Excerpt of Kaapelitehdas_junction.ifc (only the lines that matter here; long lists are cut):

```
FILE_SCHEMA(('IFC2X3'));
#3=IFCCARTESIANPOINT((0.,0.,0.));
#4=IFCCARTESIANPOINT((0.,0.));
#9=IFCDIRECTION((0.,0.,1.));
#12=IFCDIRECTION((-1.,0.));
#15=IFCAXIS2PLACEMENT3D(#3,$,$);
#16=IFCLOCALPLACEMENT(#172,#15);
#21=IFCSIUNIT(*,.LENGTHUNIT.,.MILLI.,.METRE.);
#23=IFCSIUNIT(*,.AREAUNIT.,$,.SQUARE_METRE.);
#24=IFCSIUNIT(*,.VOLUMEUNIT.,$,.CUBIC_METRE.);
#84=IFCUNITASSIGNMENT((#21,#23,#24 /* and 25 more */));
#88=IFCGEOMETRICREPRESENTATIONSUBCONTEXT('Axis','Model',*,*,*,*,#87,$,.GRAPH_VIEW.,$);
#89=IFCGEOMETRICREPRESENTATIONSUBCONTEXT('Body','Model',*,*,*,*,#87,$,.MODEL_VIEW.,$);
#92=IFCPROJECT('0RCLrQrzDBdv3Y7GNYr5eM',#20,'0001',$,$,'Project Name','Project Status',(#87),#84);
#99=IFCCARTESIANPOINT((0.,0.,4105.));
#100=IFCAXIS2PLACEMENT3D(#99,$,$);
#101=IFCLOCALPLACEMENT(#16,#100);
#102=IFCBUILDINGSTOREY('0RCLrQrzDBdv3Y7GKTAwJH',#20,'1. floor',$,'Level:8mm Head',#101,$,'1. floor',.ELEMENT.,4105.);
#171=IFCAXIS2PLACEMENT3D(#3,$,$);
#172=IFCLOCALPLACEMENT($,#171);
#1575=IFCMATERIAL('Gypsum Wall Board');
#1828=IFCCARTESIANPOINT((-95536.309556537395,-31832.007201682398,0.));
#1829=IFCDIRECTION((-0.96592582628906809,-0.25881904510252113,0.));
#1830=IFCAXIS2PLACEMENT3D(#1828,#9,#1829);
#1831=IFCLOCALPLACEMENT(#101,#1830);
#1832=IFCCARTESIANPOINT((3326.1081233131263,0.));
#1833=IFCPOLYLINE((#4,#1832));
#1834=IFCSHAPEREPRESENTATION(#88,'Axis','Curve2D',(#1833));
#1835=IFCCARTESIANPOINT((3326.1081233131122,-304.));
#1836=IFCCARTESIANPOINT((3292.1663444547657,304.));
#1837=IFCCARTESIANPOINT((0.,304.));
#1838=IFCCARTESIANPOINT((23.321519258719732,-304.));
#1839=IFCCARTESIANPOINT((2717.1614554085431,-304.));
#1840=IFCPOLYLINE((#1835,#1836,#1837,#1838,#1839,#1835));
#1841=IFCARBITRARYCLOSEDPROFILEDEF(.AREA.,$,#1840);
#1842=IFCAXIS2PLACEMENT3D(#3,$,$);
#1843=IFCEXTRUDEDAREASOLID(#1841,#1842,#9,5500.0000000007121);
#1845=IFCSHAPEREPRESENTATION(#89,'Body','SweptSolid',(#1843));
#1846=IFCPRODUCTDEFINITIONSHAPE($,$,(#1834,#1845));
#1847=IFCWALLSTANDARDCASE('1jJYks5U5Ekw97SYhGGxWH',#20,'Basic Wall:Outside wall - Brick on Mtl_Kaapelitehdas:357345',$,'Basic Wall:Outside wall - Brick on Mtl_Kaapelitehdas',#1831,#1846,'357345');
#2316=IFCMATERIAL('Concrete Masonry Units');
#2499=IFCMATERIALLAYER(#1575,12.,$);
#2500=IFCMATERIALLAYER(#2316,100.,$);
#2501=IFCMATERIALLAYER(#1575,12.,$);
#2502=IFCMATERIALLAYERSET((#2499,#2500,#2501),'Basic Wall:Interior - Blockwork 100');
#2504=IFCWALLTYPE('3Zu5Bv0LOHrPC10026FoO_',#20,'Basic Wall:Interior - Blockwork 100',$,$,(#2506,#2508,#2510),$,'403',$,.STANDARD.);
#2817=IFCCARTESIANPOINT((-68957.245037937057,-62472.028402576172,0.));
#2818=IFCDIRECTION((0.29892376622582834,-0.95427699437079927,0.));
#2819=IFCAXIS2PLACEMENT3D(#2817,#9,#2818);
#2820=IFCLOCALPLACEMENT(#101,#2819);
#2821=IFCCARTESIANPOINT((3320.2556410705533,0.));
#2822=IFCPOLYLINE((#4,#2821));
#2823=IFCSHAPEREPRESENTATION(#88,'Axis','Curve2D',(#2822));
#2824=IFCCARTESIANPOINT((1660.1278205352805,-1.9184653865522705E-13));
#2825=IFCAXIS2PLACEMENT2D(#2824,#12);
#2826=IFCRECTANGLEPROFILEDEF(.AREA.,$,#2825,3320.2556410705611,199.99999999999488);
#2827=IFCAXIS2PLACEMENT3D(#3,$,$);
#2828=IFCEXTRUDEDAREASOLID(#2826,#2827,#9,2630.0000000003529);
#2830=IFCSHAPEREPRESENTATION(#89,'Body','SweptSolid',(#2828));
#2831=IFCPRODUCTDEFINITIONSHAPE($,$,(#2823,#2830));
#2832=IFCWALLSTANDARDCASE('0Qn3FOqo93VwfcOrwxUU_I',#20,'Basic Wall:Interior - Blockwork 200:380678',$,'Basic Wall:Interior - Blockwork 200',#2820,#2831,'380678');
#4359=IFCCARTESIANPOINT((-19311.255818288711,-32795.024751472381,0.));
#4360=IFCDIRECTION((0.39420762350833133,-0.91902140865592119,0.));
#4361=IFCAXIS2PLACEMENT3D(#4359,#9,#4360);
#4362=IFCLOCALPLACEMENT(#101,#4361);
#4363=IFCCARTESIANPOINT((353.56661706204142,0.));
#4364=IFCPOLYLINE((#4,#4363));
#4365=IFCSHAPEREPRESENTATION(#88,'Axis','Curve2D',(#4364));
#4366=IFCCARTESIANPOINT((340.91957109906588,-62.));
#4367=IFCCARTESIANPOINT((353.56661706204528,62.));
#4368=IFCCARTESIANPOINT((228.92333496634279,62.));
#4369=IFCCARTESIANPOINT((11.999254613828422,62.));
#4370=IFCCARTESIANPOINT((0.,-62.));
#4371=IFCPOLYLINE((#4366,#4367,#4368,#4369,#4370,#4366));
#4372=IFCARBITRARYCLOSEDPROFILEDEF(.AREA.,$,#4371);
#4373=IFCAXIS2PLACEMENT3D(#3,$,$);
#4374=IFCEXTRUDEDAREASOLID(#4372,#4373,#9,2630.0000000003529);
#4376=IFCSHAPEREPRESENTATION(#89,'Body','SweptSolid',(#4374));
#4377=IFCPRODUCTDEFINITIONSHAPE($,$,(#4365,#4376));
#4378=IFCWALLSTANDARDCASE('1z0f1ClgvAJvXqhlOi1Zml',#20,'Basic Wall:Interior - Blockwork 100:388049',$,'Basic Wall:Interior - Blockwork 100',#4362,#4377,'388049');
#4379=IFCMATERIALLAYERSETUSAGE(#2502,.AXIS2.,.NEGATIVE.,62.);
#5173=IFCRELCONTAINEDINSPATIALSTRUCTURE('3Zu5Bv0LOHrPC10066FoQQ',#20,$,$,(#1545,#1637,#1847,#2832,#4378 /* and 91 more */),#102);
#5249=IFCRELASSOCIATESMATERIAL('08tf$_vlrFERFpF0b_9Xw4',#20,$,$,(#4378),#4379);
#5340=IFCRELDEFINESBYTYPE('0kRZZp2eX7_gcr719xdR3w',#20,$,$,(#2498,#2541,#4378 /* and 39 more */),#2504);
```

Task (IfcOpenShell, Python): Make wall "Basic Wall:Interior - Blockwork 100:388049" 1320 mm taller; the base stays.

```python
import ifcopenshell
import ifcopenshell.geom
import ifcopenshell.util.representation
import ifcopenshell.util.shape

model = ifcopenshell.open("Kaapelitehdas_junction.ifc")
settings = ifcopenshell.geom.settings()


def volume(element):
    """Net volume in cubic metres, openings subtracted."""
    shape = ifcopenshell.geom.create_shape(settings, element)
    return ifcopenshell.util.shape.get_volume(shape.geometry)


wall = model.by_guid("1z0f1ClgvAJvXqhlOi1Zml")
before = volume(wall)

body = ifcopenshell.util.representation.get_representation(wall, "Model", "Body")
solid = body.Items[0]
old_height = solid.Depth
solid.Depth += 1320.0
after = volume(wall)

print(f"height {old_height:g} -> {solid.Depth:g}, volume {before:.3f} -> {after:.3f} m3")

model.write("Kaapelitehdas_junction_rev.ifc")
```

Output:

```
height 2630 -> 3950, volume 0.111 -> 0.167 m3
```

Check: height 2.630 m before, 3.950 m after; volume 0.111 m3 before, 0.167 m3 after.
